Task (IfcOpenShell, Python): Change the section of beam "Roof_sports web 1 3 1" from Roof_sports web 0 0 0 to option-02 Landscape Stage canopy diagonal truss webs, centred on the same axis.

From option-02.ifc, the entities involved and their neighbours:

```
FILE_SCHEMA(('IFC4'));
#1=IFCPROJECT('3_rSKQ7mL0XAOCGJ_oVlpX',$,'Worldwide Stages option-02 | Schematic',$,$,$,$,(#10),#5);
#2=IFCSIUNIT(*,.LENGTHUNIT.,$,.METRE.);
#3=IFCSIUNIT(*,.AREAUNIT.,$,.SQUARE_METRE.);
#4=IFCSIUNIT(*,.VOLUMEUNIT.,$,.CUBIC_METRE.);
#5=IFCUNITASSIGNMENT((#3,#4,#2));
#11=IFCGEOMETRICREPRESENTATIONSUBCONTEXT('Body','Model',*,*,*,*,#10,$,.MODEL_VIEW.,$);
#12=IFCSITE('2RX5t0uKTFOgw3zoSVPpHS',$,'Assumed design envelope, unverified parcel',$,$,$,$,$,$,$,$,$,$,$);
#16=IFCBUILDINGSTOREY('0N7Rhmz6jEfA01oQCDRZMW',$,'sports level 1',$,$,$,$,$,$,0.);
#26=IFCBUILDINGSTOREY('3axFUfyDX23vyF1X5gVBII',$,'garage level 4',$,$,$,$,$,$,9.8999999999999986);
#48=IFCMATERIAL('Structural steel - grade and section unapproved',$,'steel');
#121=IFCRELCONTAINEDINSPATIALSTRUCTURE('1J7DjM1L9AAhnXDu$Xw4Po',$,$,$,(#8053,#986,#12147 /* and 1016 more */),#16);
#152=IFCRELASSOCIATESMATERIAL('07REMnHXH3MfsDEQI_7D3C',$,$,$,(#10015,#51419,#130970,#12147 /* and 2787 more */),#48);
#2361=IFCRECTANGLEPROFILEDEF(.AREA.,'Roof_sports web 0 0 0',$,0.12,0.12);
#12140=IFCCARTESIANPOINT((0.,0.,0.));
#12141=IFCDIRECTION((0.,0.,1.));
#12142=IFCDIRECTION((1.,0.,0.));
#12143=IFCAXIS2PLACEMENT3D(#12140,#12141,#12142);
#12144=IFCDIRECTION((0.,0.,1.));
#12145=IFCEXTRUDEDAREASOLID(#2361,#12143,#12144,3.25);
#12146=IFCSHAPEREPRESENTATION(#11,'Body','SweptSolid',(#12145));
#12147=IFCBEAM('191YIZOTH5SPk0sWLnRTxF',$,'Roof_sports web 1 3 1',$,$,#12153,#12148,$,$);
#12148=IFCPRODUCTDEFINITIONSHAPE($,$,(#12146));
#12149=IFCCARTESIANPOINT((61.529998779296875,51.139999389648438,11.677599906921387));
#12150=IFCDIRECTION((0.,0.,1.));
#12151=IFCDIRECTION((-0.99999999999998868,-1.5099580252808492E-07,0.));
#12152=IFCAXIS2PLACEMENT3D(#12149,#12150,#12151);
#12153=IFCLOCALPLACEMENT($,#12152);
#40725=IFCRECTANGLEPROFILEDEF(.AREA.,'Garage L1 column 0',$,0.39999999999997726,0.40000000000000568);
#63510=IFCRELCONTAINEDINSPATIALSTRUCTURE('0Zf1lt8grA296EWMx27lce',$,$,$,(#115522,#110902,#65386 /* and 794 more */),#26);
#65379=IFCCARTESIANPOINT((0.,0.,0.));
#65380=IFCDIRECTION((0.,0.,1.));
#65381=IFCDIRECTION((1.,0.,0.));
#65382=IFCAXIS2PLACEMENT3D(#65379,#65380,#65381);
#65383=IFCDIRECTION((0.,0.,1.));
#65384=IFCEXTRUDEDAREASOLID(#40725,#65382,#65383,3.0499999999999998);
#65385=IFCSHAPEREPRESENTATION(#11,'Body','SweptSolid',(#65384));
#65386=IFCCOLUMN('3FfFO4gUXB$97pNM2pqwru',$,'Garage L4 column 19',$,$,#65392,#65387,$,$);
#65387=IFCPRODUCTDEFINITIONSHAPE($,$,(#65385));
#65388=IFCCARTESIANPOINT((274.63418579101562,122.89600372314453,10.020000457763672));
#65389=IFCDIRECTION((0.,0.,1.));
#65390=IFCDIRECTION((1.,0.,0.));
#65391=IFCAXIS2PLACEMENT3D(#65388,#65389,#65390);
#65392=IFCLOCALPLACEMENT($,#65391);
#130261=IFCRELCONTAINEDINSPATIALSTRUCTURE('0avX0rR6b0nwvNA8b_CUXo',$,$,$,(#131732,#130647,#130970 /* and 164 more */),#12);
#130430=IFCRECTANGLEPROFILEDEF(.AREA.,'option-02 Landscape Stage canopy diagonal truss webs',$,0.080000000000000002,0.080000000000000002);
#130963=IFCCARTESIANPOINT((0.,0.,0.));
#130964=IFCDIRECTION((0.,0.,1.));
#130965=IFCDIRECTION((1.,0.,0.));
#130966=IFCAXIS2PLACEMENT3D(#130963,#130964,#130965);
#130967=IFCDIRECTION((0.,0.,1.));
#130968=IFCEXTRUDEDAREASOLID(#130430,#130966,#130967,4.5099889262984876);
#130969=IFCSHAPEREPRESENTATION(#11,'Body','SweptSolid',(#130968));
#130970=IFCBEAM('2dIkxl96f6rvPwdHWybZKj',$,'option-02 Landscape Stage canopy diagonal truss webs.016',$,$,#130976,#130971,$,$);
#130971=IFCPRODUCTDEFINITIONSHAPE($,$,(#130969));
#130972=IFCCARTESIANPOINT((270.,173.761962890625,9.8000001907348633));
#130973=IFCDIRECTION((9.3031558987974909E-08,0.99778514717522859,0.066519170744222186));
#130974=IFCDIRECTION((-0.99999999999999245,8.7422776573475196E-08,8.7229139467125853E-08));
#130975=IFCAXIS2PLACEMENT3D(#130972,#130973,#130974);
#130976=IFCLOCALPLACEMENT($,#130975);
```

```python
import ifcopenshell
import ifcopenshell.util.element
import ifcopenshell.util.representation

model = ifcopenshell.open("option-02.ifc")

member = model.by_guid("191YIZOTH5SPk0sWLnRTxF")
source = next(p for p in model.by_type("IfcRectangleProfileDef") if p.ProfileName == "option-02 Landscape Stage canopy diagonal truss webs")

body = ifcopenshell.util.representation.get_representation(member, "Model", "Body")
solid = body.Items[0]
old_profile = solid.SweptArea

# Copy the section's sizes but keep this member's own profile position.
profile = ifcopenshell.util.element.copy(model, source)
profile.Position = old_profile.Position
solid.SweptArea = profile
if not model.get_total_inverses(old_profile):
    ifcopenshell.util.element.remove_deep2(model, old_profile)

print(solid.SweptArea)

model.write("option-02_v2.ifc")
```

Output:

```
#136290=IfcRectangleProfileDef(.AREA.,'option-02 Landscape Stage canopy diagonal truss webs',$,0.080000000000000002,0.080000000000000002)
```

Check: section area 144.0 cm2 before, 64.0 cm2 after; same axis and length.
